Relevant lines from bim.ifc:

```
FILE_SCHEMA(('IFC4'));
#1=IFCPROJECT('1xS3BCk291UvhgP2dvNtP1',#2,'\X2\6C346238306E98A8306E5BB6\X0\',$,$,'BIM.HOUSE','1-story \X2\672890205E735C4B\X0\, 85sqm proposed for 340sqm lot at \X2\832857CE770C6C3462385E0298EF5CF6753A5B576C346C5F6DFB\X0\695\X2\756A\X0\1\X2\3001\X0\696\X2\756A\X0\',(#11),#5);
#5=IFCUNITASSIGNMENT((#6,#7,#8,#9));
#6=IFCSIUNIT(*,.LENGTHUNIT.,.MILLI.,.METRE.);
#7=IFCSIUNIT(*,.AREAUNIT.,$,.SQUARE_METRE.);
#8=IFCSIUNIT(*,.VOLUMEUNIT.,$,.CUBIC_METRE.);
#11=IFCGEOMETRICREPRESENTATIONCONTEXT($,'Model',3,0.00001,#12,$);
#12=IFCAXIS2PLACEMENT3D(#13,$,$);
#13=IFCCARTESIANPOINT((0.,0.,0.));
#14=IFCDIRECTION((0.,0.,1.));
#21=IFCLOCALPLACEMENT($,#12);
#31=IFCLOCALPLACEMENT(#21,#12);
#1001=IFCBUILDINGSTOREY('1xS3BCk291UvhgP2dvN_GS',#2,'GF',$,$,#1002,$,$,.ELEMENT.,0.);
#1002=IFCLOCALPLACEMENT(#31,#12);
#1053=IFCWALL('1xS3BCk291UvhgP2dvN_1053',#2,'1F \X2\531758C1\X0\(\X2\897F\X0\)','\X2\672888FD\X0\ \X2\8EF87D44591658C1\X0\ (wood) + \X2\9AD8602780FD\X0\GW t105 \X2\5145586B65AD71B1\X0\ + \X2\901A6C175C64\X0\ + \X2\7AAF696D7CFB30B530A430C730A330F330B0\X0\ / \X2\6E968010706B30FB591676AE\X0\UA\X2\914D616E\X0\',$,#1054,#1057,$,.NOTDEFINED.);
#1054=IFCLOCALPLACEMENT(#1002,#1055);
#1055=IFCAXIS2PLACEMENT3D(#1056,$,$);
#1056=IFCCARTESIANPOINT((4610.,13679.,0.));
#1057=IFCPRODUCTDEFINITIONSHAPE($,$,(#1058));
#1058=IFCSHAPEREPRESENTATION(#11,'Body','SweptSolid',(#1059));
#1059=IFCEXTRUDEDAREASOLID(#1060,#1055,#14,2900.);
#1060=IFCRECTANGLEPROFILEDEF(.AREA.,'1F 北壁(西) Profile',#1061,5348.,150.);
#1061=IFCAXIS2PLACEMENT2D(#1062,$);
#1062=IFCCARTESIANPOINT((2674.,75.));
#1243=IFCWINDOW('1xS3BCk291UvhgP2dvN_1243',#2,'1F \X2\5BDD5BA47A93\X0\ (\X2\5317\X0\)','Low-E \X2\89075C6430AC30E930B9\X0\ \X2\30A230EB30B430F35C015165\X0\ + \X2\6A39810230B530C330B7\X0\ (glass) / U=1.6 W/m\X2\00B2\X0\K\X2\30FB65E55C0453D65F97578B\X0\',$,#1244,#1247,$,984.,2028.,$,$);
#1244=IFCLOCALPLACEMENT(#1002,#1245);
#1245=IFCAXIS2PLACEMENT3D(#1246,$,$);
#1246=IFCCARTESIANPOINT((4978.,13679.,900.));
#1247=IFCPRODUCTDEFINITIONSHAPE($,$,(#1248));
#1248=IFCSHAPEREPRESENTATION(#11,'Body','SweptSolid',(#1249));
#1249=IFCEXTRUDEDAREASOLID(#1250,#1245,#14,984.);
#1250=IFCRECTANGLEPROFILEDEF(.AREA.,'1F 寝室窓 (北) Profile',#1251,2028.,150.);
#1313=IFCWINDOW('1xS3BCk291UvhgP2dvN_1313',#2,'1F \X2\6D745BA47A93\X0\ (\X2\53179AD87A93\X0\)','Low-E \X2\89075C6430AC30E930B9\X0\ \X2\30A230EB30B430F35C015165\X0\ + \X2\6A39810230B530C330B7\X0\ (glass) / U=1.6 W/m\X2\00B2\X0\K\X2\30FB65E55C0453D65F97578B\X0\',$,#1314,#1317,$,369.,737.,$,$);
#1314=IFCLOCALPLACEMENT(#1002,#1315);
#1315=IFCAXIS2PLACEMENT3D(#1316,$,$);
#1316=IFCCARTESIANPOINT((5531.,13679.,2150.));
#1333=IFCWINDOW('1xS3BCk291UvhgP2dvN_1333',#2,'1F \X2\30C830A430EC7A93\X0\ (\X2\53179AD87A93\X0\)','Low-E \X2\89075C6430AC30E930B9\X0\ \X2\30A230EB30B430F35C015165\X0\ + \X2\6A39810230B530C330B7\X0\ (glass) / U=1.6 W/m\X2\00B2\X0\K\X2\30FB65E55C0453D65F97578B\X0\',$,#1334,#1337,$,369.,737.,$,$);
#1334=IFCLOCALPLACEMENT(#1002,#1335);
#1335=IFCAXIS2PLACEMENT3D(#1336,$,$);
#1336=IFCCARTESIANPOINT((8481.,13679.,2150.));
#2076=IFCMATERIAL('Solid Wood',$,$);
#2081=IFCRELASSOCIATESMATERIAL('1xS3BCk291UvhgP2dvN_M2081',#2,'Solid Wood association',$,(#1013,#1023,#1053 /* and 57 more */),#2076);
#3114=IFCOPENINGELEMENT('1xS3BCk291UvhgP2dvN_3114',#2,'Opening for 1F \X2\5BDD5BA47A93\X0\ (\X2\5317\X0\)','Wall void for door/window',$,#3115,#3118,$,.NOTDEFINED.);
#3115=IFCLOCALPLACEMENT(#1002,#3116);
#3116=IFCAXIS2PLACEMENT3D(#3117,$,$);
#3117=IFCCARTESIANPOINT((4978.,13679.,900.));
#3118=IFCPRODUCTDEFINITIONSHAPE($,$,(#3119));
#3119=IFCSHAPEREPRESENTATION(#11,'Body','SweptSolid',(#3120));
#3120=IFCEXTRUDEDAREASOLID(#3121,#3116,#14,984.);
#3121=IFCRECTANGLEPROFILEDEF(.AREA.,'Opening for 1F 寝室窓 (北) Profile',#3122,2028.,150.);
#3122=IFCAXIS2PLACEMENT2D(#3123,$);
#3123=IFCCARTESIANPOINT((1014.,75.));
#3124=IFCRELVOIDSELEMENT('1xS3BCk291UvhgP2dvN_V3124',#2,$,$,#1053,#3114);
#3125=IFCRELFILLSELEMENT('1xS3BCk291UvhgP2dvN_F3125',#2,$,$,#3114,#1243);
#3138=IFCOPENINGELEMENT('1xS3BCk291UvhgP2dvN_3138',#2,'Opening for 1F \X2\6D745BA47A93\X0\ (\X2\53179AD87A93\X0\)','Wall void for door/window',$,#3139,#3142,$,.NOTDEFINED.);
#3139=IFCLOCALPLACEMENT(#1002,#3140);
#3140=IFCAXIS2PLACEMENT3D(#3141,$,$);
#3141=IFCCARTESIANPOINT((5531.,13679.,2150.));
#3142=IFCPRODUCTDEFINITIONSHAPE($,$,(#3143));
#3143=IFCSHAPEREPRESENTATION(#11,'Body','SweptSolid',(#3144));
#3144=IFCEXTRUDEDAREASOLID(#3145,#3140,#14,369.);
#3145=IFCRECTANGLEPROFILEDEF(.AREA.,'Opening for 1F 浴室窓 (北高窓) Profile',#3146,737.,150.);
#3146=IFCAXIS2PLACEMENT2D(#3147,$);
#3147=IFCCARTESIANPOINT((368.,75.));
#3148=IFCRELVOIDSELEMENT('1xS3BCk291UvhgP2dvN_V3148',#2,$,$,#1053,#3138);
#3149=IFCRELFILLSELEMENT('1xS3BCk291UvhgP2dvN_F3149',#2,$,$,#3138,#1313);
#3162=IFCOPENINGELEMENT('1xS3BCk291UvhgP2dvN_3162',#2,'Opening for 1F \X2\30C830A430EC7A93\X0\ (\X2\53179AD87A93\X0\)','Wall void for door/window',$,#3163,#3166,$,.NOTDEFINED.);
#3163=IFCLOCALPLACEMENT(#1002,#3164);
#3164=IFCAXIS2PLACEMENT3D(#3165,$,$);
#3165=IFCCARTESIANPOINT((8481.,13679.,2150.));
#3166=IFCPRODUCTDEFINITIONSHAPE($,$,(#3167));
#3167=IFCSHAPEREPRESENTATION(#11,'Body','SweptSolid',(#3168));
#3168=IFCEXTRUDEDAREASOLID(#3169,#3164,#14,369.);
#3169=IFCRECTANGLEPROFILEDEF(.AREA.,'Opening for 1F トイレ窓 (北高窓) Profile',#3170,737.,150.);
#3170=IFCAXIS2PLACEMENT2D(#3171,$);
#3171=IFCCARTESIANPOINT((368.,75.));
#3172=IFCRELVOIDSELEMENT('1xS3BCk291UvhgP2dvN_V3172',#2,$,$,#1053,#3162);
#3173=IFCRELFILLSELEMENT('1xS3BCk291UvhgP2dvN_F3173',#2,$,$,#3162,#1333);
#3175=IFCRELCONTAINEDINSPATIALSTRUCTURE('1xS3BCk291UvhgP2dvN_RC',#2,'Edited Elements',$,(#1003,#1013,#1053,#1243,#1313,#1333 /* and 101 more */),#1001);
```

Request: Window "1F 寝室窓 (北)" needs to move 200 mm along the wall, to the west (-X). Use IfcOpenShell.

```python
import ifcopenshell
import ifcopenshell.api.geometry
import ifcopenshell.util.placement
import ifcopenshell.util.unit

model = ifcopenshell.open("bim.ifc")
unit_scale = ifcopenshell.util.unit.calculate_unit_scale(model)

window = model.by_id(1243)
opening = window.FillsVoids[0].RelatingOpeningElement
wall = opening.VoidsElements[0].RelatingBuildingElement

wall_matrix = ifcopenshell.util.placement.get_local_placement(wall.ObjectPlacement)
shift = wall_matrix[:3, 0] * -0.2 / unit_scale
before = ifcopenshell.util.placement.get_local_placement(window.ObjectPlacement)[:3, 3].copy()

# The window is not placed relative to its opening, so move both.
for product in (opening, window):
    matrix = ifcopenshell.util.placement.get_local_placement(product.ObjectPlacement)
    matrix[:3, 3] += shift
    ifcopenshell.api.geometry.edit_object_placement(model, product=product, matrix=matrix, is_si=False)

after = ifcopenshell.util.placement.get_local_placement(window.ObjectPlacement)[:3, 3]
print("window moved by", (after - before).round(3) + 0.0)

model.write("bim-out.ifc")
```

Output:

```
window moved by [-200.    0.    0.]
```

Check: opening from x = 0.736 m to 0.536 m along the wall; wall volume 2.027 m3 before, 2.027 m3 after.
